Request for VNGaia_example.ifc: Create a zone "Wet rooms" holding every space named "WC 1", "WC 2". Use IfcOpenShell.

First a look at what the model holds.

```python
import ifcopenshell

model = ifcopenshell.open("VNGaia_example.ifc")
print(model.schema)
seen = {}
for space in model.by_type("IfcSpace"):
    seen[space.LongName] = seen.get(space.LongName, 0) + 1
for name, count in sorted(seen.items(), key=str):
    print(count, "x", name)
print("zones:", [z.Name for z in model.by_type("IfcZone")][:20])
```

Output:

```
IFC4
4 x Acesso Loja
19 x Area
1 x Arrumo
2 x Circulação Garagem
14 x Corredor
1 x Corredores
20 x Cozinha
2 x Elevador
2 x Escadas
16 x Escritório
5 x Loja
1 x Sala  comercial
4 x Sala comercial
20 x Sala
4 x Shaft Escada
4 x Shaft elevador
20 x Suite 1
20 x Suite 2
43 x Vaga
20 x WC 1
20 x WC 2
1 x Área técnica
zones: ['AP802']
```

```python
import ifcopenshell
import ifcopenshell.api.group
import ifcopenshell.api.root

model = ifcopenshell.open("VNGaia_example.ifc")

names = {"WC 1", "WC 2"}
spaces = [s for s in model.by_type("IfcSpace") if s.LongName in names]

zone = ifcopenshell.api.root.create_entity(model, ifc_class="IfcZone", name="Wet rooms")
ifcopenshell.api.group.assign_group(model, products=spaces, group=zone)
print(len(spaces), "spaces in", zone.Name)

model.write("VNGaia_example_rev.ifc")
```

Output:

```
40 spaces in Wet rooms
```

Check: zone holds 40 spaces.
